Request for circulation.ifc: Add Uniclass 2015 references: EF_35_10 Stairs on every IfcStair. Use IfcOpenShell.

First a look at what the model holds.

```python
import ifcopenshell

model = ifcopenshell.open("circulation.ifc")
print(model.schema)
print("classifications:", [c.Name for c in model.by_type("IfcClassification")])
for ifc_class in ("IfcDoor", "IfcRoof", "IfcStair", "IfcWall", "IfcWindow"):
    print(ifc_class, len(model.by_type(ifc_class)))
```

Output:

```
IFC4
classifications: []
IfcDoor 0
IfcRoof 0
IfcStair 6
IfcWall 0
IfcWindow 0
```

```python
import ifcopenshell
import ifcopenshell.api.classification

model = ifcopenshell.open("circulation.ifc")

system = ifcopenshell.api.classification.add_classification(model, classification="Uniclass 2015")

codes = {
    "IfcStair": ("EF_35_10", "Stairs"),
}
for ifc_class, (code, name) in codes.items():
    products = model.by_type(ifc_class)
    ifcopenshell.api.classification.add_reference(
        model, products=products, classification=system, identification=code, name=name
    )
    print(code, len(products))

model.write("circulation_v2.ifc")
```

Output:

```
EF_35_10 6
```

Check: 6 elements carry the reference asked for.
